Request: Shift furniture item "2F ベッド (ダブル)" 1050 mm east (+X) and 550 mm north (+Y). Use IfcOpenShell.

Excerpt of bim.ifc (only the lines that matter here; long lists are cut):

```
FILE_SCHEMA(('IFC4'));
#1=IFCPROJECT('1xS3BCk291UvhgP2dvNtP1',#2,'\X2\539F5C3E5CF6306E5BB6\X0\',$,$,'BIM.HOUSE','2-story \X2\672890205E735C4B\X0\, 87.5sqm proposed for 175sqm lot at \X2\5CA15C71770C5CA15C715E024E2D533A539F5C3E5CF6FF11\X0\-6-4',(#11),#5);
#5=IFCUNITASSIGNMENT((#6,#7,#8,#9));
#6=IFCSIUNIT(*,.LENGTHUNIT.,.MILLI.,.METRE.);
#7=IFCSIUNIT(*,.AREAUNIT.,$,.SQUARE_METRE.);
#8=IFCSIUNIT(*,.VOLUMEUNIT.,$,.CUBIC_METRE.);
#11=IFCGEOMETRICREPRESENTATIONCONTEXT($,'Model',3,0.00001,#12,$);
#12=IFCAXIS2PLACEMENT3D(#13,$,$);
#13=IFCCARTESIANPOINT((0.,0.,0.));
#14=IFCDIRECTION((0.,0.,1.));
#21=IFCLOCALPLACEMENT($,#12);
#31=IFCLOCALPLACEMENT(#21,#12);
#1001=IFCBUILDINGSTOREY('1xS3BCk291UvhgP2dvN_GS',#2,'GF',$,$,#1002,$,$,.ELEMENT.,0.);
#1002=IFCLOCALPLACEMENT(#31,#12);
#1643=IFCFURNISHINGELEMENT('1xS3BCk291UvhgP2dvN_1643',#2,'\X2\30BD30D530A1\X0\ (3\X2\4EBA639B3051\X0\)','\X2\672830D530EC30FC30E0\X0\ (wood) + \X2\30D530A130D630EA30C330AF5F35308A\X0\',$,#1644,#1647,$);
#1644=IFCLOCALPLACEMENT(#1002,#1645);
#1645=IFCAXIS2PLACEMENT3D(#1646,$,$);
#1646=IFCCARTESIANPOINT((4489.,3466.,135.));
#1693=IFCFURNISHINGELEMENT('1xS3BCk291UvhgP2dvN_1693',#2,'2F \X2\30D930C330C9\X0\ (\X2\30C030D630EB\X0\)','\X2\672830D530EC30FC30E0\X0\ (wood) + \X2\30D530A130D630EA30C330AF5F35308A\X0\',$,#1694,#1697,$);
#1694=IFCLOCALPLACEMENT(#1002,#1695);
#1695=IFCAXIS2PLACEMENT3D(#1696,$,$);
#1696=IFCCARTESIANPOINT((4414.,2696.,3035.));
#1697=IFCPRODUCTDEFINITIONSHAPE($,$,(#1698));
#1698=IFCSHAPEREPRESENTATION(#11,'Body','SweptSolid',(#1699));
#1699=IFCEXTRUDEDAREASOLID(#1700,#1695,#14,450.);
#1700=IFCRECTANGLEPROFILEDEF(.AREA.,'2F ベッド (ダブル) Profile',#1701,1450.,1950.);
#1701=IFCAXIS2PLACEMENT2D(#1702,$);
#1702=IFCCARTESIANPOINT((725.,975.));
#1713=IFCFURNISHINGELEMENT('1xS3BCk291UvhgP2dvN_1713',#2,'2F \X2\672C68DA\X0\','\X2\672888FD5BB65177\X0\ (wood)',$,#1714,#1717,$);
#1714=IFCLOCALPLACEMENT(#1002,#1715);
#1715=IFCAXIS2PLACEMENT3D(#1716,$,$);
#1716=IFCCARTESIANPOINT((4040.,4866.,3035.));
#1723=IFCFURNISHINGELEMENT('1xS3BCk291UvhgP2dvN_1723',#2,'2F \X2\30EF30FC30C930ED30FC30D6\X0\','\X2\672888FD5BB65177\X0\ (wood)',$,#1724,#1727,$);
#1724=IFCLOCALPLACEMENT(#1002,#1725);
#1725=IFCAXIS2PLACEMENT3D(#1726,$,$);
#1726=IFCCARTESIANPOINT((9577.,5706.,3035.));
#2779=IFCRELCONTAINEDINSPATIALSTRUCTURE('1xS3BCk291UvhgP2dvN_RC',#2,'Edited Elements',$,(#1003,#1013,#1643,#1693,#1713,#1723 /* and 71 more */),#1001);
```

```python
import ifcopenshell
import ifcopenshell.api.geometry
import ifcopenshell.util.placement
import ifcopenshell.util.unit

model = ifcopenshell.open("bim.ifc")
unit_scale = ifcopenshell.util.unit.calculate_unit_scale(model)

item = model.by_id(1693)
matrix = ifcopenshell.util.placement.get_local_placement(item.ObjectPlacement)
matrix[0, 3] += 1.05 / unit_scale
matrix[1, 3] += 0.55 / unit_scale
ifcopenshell.api.geometry.edit_object_placement(model, product=item, matrix=matrix, is_si=False)

print(ifcopenshell.util.placement.get_local_placement(item.ObjectPlacement).round(3) + 0.0)

model.write("bim-out.ifc")
```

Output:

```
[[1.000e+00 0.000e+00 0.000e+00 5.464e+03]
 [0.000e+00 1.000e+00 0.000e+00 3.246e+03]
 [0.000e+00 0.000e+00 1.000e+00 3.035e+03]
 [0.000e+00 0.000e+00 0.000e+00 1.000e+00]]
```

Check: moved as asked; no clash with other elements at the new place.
